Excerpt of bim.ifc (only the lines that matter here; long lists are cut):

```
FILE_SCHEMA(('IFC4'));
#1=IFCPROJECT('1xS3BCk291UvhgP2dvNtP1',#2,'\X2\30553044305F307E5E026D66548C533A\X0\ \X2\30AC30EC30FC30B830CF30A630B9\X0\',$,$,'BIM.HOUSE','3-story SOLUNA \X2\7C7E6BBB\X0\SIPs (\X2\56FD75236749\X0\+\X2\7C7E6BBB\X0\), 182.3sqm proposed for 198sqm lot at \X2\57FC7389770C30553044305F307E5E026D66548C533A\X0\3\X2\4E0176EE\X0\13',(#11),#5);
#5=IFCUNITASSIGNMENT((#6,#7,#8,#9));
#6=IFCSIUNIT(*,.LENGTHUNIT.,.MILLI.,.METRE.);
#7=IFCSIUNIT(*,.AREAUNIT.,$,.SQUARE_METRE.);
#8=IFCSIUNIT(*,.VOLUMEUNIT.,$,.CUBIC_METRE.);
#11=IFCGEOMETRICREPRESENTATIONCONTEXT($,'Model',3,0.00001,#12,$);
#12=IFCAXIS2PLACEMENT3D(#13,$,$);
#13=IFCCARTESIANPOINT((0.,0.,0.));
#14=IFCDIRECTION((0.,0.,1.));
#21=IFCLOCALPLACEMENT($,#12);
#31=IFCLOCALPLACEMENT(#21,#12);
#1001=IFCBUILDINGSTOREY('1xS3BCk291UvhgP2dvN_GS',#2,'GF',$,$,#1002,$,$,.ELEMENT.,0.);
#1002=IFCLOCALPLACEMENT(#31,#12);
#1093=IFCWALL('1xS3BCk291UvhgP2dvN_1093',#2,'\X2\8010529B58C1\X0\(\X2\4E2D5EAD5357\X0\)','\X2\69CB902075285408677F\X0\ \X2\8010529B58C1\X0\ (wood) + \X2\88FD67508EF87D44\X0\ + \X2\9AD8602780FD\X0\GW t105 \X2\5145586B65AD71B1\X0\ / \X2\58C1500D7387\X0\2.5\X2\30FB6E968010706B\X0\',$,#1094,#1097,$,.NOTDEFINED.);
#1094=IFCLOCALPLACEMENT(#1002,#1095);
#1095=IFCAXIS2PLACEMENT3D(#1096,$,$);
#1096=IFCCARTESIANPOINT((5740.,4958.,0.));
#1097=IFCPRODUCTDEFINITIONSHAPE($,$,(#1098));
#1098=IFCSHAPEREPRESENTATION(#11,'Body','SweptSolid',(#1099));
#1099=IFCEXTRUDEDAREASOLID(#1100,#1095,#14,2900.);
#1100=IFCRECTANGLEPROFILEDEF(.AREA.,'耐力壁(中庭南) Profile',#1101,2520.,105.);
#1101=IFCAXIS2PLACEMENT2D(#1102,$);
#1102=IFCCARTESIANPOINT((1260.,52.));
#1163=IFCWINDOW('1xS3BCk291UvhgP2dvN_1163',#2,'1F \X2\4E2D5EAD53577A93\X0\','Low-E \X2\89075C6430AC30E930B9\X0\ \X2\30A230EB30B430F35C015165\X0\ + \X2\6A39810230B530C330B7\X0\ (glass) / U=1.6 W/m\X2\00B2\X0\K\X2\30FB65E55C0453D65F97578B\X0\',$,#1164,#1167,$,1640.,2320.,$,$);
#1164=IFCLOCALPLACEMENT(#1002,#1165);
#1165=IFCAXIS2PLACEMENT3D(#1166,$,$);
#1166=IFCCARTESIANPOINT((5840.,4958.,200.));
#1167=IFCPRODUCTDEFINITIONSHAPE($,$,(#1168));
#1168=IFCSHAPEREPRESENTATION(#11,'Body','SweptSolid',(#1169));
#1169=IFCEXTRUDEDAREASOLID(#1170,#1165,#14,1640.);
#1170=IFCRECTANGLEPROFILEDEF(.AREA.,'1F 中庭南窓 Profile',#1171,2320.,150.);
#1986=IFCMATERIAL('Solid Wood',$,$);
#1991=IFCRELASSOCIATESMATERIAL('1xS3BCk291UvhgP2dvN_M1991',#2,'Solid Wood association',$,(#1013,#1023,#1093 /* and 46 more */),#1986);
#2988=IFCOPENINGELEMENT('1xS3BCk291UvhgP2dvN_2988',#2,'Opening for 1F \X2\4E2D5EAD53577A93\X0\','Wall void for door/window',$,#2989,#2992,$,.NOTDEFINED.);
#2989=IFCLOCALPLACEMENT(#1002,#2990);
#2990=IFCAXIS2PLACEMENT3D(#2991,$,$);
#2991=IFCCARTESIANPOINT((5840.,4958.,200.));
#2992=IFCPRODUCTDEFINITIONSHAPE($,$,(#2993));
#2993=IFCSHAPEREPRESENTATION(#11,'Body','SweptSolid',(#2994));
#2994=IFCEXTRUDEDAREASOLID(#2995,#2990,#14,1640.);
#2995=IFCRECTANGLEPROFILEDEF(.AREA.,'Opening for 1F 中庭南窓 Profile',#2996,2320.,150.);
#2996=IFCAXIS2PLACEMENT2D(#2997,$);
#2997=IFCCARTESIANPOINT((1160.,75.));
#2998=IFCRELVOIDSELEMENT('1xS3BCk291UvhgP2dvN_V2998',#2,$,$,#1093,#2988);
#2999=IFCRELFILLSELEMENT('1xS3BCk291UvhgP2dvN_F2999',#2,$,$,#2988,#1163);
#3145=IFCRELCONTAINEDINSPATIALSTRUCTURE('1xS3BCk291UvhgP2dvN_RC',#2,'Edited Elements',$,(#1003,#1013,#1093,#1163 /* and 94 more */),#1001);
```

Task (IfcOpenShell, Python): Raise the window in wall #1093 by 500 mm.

```python
import numpy as np
import ifcopenshell
import ifcopenshell.api.geometry
import ifcopenshell.util.placement
import ifcopenshell.util.unit

model = ifcopenshell.open("bim.ifc")
unit_scale = ifcopenshell.util.unit.calculate_unit_scale(model)

window = model.by_guid("1xS3BCk291UvhgP2dvN_1163")
opening = window.FillsVoids[0].RelatingOpeningElement
dz = 0.5 / unit_scale

shift = np.array([0.0, 0.0, dz])
# The window is not placed relative to its opening, so move both.
for product in (opening, window):
    matrix = ifcopenshell.util.placement.get_local_placement(product.ObjectPlacement)
    matrix[:3, 3] += shift
    ifcopenshell.api.geometry.edit_object_placement(model, product=product, matrix=matrix, is_si=False)

print(f"moved by {dz * unit_scale:+.3f} m")

model.write("bim_rev.ifc")
```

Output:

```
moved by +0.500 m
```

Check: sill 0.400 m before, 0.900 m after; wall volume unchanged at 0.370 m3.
